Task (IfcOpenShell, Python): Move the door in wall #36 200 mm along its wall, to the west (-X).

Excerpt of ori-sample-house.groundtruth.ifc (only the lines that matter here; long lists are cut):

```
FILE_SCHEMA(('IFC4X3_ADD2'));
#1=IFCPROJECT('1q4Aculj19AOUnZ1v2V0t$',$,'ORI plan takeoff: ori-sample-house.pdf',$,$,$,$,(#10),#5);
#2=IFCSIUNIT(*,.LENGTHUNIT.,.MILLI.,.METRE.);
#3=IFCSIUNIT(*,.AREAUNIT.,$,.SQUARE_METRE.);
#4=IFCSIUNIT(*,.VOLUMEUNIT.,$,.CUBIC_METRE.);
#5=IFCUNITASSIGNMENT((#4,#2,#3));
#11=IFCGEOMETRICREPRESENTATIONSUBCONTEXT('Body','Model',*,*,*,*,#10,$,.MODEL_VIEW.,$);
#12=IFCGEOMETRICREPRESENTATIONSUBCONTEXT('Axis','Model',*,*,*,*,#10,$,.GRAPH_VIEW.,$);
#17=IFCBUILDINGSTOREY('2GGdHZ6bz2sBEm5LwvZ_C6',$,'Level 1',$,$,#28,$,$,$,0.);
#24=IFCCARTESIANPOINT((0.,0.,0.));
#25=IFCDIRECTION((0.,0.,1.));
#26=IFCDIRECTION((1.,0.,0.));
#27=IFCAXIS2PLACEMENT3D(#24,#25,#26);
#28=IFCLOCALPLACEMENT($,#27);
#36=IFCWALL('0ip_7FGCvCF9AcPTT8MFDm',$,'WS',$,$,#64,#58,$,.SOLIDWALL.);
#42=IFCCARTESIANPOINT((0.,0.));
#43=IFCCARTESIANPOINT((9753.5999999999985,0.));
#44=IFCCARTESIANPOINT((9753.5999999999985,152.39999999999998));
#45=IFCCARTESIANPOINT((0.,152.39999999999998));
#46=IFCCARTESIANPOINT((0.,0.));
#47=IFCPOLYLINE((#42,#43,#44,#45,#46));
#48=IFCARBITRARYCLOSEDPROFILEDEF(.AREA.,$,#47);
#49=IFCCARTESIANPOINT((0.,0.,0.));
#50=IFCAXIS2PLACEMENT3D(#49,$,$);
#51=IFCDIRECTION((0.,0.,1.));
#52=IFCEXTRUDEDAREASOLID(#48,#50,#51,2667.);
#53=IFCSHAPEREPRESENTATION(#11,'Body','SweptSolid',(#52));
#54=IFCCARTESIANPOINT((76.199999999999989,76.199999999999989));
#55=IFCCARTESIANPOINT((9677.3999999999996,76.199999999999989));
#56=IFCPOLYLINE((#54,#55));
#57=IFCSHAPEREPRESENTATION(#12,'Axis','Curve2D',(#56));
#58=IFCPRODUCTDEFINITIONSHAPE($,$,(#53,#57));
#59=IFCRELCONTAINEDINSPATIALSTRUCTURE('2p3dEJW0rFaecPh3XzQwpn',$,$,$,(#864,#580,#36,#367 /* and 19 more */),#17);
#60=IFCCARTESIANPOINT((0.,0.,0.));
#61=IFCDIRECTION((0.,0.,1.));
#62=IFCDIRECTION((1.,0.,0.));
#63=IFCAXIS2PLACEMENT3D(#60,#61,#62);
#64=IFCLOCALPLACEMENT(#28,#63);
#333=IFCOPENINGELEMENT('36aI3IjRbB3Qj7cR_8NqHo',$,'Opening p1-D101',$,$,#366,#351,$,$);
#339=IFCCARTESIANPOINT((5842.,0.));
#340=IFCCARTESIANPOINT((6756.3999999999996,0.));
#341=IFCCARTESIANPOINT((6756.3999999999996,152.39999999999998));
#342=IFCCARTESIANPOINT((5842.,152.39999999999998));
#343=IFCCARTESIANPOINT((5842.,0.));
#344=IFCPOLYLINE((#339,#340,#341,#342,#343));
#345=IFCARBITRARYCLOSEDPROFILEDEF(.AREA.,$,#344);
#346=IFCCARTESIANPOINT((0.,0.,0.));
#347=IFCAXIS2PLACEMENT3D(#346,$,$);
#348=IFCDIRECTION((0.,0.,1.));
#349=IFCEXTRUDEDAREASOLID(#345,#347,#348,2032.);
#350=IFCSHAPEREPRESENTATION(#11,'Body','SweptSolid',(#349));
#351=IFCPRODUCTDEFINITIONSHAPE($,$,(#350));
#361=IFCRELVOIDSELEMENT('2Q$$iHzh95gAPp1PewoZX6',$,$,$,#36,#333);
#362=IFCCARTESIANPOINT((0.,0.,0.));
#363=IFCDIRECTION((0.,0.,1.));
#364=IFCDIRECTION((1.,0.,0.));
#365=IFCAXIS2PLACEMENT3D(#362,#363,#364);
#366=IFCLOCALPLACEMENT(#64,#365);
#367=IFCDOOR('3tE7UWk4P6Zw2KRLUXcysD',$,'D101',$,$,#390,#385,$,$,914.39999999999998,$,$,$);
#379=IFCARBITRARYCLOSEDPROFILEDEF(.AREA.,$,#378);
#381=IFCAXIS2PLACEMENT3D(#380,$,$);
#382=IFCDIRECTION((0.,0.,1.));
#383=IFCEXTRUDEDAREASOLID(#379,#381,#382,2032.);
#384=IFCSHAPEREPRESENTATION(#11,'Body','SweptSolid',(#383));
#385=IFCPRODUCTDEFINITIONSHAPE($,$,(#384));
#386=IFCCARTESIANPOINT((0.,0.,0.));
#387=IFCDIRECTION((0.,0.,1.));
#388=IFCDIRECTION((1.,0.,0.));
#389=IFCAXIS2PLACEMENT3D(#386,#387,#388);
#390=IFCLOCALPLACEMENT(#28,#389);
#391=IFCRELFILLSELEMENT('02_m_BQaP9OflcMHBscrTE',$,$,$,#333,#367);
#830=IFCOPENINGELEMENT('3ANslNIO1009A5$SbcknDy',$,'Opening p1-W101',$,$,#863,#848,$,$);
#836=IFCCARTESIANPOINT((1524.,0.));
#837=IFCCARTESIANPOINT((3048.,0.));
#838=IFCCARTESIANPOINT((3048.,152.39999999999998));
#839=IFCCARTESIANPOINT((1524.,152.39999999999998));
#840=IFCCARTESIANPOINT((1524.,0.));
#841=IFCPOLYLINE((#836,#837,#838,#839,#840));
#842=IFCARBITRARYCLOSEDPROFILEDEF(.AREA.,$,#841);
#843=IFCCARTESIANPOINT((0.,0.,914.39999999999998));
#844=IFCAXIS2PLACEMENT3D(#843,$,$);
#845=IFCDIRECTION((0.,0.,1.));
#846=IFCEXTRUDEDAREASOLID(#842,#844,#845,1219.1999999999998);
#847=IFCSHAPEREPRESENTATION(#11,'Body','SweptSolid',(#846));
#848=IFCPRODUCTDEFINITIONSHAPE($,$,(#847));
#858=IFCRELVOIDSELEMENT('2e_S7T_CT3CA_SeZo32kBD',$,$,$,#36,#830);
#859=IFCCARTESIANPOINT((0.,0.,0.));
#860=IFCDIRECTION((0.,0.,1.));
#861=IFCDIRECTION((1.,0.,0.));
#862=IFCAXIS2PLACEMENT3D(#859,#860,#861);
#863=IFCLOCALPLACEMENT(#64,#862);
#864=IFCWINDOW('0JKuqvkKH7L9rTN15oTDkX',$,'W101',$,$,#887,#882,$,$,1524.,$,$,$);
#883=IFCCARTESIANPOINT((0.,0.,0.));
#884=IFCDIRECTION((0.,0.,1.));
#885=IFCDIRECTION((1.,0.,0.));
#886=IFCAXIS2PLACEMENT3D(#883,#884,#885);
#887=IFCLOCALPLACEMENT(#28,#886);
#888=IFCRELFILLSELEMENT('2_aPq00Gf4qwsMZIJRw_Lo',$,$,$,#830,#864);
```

```python
import ifcopenshell
import ifcopenshell.api.geometry
import ifcopenshell.util.placement
import ifcopenshell.util.unit

model = ifcopenshell.open("ori-sample-house.groundtruth.ifc")
unit_scale = ifcopenshell.util.unit.calculate_unit_scale(model)

door = model.by_guid("3tE7UWk4P6Zw2KRLUXcysD")
opening = door.FillsVoids[0].RelatingOpeningElement
wall = opening.VoidsElements[0].RelatingBuildingElement

wall_matrix = ifcopenshell.util.placement.get_local_placement(wall.ObjectPlacement)
shift = wall_matrix[:3, 0] * -0.2 / unit_scale
before = ifcopenshell.util.placement.get_local_placement(door.ObjectPlacement)[:3, 3].copy()

# The door is not placed relative to its opening, so move both.
for product in (opening, door):
    matrix = ifcopenshell.util.placement.get_local_placement(product.ObjectPlacement)
    matrix[:3, 3] += shift
    ifcopenshell.api.geometry.edit_object_placement(model, product=product, matrix=matrix, is_si=False)

after = ifcopenshell.util.placement.get_local_placement(door.ObjectPlacement)[:3, 3]
print("door moved by", (after - before).round(3) + 0.0)

model.write("ori-sample-house.groundtruth-out.ifc")
```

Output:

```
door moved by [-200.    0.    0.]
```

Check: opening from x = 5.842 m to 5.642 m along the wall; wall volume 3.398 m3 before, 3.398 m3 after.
